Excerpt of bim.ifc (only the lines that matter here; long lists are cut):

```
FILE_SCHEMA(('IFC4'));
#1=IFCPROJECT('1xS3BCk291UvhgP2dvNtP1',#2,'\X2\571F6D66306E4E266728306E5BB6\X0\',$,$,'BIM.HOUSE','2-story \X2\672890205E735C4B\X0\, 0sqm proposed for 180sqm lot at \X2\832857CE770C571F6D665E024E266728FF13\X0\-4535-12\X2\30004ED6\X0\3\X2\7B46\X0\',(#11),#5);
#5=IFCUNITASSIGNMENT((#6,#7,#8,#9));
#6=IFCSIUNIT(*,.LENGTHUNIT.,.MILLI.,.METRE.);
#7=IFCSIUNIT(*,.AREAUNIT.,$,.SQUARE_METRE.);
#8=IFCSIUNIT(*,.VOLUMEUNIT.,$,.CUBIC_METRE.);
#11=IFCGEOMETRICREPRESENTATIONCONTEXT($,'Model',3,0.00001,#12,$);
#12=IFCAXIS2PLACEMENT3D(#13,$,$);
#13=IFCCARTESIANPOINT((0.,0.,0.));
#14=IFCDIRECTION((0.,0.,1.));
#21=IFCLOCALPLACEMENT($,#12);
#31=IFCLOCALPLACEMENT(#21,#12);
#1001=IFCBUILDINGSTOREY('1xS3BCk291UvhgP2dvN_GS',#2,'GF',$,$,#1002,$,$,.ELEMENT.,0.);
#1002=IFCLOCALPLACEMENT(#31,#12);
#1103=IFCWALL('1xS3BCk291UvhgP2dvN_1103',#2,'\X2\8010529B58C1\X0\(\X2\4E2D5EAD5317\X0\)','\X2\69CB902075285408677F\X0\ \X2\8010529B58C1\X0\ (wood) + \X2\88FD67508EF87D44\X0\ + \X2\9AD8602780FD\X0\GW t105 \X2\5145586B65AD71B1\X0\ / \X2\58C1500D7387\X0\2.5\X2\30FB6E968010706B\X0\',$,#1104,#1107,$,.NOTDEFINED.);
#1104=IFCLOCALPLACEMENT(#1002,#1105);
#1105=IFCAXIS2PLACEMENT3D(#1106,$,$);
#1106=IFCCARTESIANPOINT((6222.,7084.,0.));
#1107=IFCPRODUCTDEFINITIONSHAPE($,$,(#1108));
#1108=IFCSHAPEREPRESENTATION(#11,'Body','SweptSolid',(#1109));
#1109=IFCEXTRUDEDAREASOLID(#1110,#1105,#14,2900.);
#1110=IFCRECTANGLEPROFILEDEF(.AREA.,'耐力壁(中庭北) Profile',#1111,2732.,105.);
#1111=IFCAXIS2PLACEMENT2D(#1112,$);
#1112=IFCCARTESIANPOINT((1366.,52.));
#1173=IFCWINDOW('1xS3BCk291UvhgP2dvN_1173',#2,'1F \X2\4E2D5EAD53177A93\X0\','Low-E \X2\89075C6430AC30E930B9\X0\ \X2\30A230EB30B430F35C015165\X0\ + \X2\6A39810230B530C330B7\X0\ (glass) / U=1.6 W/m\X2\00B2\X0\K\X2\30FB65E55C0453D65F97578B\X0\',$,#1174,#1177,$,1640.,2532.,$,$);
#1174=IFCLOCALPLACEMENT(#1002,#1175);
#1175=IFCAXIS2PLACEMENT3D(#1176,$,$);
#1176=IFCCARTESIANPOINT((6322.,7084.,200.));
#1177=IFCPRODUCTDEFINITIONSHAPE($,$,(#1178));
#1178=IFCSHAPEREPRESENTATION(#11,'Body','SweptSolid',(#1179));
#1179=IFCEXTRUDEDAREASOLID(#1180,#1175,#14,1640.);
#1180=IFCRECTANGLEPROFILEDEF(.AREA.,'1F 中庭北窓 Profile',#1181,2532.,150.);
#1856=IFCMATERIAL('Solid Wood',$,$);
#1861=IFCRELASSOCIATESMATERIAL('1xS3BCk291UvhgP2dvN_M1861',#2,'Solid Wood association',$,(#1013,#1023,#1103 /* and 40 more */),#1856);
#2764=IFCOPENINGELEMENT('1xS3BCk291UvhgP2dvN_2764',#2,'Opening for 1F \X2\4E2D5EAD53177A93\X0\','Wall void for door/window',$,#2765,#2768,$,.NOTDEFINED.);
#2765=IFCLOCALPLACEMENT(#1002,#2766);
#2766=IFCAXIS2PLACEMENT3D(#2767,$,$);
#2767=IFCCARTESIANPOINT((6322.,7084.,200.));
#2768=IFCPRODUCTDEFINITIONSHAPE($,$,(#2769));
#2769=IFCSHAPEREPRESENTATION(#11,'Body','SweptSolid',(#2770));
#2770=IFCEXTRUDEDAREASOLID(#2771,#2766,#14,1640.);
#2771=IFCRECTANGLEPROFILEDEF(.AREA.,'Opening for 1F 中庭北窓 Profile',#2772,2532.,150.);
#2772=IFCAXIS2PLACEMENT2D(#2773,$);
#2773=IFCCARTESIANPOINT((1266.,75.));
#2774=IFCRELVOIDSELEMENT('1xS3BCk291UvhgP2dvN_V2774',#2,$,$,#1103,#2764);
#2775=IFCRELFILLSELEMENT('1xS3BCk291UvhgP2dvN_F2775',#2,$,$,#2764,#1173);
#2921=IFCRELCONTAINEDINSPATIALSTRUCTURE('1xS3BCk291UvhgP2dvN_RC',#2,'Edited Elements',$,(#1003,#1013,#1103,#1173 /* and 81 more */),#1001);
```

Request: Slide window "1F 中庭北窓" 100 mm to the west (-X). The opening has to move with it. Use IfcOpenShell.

```python
import ifcopenshell
import ifcopenshell.api.geometry
import ifcopenshell.util.placement

model = ifcopenshell.open("bim.ifc")

window = model.by_id(1173)
opening = window.FillsVoids[0].RelatingOpeningElement
wall = opening.VoidsElements[0].RelatingBuildingElement

wall_matrix = ifcopenshell.util.placement.get_local_placement(wall.ObjectPlacement)
shift = wall_matrix[:3, 0] * -100.0
before = ifcopenshell.util.placement.get_local_placement(window.ObjectPlacement)[:3, 3].copy()

# The window is not placed relative to its opening, so move both.
for product in (opening, window):
    matrix = ifcopenshell.util.placement.get_local_placement(product.ObjectPlacement)
    matrix[:3, 3] += shift
    ifcopenshell.api.geometry.edit_object_placement(model, product=product, matrix=matrix, is_si=False)

after = ifcopenshell.util.placement.get_local_placement(window.ObjectPlacement)[:3, 3]
print("window moved by", (after - before).round(3) + 0.0)

model.write("bim_updated.ifc")
```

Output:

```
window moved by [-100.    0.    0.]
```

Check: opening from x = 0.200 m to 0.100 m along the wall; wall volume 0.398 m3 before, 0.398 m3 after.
